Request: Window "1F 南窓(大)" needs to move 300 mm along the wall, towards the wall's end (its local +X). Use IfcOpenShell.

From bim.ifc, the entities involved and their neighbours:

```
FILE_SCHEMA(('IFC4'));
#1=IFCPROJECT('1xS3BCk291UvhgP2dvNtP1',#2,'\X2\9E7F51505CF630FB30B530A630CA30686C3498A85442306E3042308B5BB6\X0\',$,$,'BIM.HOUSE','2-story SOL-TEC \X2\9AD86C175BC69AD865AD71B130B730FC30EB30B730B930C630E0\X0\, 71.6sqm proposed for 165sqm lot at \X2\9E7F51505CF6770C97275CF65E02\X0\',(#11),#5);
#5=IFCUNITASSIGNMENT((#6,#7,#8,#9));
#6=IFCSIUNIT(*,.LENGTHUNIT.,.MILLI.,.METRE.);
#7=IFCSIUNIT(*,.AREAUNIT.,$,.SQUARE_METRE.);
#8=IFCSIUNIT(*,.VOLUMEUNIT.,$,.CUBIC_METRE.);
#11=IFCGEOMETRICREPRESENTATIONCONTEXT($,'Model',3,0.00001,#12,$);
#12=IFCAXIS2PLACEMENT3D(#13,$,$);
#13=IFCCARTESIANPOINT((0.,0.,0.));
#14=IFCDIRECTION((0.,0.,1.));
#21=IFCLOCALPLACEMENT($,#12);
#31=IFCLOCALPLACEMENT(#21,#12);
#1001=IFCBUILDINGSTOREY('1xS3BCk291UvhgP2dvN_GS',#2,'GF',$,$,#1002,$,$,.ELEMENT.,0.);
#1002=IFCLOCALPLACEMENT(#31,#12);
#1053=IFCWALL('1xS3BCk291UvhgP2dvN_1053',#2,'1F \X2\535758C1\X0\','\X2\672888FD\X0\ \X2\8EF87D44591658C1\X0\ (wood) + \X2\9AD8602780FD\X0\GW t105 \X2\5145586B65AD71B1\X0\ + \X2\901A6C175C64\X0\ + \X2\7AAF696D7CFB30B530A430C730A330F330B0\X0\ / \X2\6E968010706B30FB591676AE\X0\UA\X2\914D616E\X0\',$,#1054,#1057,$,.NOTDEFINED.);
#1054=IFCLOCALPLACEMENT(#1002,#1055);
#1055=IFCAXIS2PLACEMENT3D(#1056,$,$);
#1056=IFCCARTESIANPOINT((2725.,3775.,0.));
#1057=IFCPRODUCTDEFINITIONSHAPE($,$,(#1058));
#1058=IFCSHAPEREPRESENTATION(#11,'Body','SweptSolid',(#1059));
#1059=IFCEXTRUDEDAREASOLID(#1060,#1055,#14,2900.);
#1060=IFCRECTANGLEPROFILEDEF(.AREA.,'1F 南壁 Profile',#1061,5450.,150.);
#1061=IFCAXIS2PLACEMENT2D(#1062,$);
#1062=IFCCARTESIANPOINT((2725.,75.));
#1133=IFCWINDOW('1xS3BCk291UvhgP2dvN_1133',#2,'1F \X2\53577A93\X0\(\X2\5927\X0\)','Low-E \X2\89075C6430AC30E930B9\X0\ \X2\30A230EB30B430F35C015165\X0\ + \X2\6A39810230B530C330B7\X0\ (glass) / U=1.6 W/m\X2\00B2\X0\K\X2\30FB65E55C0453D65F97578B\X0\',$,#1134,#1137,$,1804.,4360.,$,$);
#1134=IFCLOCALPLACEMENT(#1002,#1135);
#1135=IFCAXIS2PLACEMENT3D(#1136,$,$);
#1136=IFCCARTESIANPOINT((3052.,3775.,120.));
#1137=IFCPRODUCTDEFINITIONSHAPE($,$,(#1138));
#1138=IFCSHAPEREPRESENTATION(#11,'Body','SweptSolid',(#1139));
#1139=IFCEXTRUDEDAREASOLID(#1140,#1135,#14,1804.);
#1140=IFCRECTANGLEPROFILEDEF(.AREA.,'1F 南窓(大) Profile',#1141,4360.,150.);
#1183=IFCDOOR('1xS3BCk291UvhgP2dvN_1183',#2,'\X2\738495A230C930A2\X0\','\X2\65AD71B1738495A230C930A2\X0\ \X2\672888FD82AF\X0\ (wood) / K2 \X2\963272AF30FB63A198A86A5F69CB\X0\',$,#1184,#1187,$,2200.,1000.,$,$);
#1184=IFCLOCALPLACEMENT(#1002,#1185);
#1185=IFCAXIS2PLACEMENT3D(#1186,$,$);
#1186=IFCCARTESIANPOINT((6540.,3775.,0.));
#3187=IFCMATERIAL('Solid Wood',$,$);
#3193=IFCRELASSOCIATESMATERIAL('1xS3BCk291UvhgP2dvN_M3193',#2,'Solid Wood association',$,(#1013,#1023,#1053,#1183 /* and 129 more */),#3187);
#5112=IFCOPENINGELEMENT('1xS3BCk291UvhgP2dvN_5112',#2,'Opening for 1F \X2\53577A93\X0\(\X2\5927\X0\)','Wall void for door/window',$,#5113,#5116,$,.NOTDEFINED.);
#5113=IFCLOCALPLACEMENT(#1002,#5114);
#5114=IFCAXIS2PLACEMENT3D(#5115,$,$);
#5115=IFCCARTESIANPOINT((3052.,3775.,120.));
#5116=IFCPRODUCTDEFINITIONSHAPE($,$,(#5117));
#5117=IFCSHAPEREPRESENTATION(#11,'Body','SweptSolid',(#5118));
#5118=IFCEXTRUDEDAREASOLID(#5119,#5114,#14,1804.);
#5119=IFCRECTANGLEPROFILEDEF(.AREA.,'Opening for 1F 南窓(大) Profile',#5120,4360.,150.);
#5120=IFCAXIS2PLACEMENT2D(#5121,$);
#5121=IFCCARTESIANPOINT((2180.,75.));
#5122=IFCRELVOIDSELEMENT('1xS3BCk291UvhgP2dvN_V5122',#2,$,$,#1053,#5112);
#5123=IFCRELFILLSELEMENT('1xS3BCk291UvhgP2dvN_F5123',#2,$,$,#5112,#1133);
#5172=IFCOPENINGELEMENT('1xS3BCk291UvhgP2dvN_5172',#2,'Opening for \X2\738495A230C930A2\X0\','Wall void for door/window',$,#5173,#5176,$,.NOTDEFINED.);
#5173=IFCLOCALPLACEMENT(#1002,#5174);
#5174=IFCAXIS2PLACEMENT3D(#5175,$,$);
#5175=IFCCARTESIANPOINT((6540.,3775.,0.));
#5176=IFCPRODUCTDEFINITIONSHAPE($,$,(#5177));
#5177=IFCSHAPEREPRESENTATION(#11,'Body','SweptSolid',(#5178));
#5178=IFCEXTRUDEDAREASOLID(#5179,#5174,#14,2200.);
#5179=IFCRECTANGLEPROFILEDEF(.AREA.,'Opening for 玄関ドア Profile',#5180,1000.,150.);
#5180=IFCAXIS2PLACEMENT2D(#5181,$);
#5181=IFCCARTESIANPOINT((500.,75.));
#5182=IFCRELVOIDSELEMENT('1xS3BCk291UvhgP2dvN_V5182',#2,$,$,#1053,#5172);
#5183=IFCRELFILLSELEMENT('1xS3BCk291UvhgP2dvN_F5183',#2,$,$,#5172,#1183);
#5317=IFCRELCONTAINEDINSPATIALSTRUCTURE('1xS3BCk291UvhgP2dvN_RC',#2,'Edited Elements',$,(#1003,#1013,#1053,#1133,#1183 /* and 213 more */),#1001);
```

```python
import ifcopenshell
import ifcopenshell.api.geometry
import ifcopenshell.util.placement
import ifcopenshell.util.unit

model = ifcopenshell.open("bim.ifc")
unit_scale = ifcopenshell.util.unit.calculate_unit_scale(model)

window = model.by_guid("1xS3BCk291UvhgP2dvN_1133")
opening = window.FillsVoids[0].RelatingOpeningElement
wall = opening.VoidsElements[0].RelatingBuildingElement

wall_matrix = ifcopenshell.util.placement.get_local_placement(wall.ObjectPlacement)
shift = wall_matrix[:3, 0] * 0.3 / unit_scale
before = ifcopenshell.util.placement.get_local_placement(window.ObjectPlacement)[:3, 3].copy()

# The window is not placed relative to its opening, so move both.
for product in (opening, window):
    matrix = ifcopenshell.util.placement.get_local_placement(product.ObjectPlacement)
    matrix[:3, 3] += shift
    ifcopenshell.api.geometry.edit_object_placement(model, product=product, matrix=matrix, is_si=False)

after = ifcopenshell.util.placement.get_local_placement(window.ObjectPlacement)[:3, 3]
print("window moved by", (after - before).round(3) + 0.0)

model.write("bim_edited.ifc")
```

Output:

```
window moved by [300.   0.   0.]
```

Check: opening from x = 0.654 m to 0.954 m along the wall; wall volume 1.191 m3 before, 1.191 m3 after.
